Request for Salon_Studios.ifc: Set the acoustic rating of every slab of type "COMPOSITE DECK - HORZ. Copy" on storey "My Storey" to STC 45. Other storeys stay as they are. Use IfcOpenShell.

First a look at what the model holds.

```python
import ifcopenshell
import ifcopenshell.util.element

model = ifcopenshell.open("Salon_Studios.ifc")
print(model.schema)
storey = next(s for s in model.by_type("IfcBuildingStorey") if s.Name == "My Storey")
slabs = [e for e in ifcopenshell.util.element.get_decomposition(storey) if e.is_a("IfcSlab")]
seen = {}
for e in slabs:
    element_type = ifcopenshell.util.element.get_type(e)
    key = (element_type.Name if element_type != e and element_type else None, ifcopenshell.util.element.get_pset(e, "Pset_SlabCommon", "AcousticRating"))
    seen[key] = seen.get(key, 0) + 1
for (name, value), count in sorted(seen.items(), key=str):
    print(count, "x", name, "|", value)
```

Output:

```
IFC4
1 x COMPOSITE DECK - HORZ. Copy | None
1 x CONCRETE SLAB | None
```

```python
import ifcopenshell
import ifcopenshell.api.pset
import ifcopenshell.util.element

model = ifcopenshell.open("Salon_Studios.ifc")

storey = next(s for s in model.by_type("IfcBuildingStorey") if s.Name == "My Storey")
slabs = [e for e in ifcopenshell.util.element.get_decomposition(storey) if e.is_a("IfcSlab")]

count = 0
for e in slabs:
    element_type = ifcopenshell.util.element.get_type(e)
    if element_type in (None, e) or element_type.Name != "COMPOSITE DECK - HORZ. Copy":
        continue
    # add_pset returns the element's existing set when there is one.
    pset = ifcopenshell.api.pset.add_pset(model, product=e, name="Pset_SlabCommon")
    ifcopenshell.api.pset.edit_pset(model, pset=pset, properties={"AcousticRating": "STC 45"})
    count += 1

print(count, "slabs updated")

model.write("Salon_Studios_v2.ifc")
```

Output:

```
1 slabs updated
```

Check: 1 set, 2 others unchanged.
